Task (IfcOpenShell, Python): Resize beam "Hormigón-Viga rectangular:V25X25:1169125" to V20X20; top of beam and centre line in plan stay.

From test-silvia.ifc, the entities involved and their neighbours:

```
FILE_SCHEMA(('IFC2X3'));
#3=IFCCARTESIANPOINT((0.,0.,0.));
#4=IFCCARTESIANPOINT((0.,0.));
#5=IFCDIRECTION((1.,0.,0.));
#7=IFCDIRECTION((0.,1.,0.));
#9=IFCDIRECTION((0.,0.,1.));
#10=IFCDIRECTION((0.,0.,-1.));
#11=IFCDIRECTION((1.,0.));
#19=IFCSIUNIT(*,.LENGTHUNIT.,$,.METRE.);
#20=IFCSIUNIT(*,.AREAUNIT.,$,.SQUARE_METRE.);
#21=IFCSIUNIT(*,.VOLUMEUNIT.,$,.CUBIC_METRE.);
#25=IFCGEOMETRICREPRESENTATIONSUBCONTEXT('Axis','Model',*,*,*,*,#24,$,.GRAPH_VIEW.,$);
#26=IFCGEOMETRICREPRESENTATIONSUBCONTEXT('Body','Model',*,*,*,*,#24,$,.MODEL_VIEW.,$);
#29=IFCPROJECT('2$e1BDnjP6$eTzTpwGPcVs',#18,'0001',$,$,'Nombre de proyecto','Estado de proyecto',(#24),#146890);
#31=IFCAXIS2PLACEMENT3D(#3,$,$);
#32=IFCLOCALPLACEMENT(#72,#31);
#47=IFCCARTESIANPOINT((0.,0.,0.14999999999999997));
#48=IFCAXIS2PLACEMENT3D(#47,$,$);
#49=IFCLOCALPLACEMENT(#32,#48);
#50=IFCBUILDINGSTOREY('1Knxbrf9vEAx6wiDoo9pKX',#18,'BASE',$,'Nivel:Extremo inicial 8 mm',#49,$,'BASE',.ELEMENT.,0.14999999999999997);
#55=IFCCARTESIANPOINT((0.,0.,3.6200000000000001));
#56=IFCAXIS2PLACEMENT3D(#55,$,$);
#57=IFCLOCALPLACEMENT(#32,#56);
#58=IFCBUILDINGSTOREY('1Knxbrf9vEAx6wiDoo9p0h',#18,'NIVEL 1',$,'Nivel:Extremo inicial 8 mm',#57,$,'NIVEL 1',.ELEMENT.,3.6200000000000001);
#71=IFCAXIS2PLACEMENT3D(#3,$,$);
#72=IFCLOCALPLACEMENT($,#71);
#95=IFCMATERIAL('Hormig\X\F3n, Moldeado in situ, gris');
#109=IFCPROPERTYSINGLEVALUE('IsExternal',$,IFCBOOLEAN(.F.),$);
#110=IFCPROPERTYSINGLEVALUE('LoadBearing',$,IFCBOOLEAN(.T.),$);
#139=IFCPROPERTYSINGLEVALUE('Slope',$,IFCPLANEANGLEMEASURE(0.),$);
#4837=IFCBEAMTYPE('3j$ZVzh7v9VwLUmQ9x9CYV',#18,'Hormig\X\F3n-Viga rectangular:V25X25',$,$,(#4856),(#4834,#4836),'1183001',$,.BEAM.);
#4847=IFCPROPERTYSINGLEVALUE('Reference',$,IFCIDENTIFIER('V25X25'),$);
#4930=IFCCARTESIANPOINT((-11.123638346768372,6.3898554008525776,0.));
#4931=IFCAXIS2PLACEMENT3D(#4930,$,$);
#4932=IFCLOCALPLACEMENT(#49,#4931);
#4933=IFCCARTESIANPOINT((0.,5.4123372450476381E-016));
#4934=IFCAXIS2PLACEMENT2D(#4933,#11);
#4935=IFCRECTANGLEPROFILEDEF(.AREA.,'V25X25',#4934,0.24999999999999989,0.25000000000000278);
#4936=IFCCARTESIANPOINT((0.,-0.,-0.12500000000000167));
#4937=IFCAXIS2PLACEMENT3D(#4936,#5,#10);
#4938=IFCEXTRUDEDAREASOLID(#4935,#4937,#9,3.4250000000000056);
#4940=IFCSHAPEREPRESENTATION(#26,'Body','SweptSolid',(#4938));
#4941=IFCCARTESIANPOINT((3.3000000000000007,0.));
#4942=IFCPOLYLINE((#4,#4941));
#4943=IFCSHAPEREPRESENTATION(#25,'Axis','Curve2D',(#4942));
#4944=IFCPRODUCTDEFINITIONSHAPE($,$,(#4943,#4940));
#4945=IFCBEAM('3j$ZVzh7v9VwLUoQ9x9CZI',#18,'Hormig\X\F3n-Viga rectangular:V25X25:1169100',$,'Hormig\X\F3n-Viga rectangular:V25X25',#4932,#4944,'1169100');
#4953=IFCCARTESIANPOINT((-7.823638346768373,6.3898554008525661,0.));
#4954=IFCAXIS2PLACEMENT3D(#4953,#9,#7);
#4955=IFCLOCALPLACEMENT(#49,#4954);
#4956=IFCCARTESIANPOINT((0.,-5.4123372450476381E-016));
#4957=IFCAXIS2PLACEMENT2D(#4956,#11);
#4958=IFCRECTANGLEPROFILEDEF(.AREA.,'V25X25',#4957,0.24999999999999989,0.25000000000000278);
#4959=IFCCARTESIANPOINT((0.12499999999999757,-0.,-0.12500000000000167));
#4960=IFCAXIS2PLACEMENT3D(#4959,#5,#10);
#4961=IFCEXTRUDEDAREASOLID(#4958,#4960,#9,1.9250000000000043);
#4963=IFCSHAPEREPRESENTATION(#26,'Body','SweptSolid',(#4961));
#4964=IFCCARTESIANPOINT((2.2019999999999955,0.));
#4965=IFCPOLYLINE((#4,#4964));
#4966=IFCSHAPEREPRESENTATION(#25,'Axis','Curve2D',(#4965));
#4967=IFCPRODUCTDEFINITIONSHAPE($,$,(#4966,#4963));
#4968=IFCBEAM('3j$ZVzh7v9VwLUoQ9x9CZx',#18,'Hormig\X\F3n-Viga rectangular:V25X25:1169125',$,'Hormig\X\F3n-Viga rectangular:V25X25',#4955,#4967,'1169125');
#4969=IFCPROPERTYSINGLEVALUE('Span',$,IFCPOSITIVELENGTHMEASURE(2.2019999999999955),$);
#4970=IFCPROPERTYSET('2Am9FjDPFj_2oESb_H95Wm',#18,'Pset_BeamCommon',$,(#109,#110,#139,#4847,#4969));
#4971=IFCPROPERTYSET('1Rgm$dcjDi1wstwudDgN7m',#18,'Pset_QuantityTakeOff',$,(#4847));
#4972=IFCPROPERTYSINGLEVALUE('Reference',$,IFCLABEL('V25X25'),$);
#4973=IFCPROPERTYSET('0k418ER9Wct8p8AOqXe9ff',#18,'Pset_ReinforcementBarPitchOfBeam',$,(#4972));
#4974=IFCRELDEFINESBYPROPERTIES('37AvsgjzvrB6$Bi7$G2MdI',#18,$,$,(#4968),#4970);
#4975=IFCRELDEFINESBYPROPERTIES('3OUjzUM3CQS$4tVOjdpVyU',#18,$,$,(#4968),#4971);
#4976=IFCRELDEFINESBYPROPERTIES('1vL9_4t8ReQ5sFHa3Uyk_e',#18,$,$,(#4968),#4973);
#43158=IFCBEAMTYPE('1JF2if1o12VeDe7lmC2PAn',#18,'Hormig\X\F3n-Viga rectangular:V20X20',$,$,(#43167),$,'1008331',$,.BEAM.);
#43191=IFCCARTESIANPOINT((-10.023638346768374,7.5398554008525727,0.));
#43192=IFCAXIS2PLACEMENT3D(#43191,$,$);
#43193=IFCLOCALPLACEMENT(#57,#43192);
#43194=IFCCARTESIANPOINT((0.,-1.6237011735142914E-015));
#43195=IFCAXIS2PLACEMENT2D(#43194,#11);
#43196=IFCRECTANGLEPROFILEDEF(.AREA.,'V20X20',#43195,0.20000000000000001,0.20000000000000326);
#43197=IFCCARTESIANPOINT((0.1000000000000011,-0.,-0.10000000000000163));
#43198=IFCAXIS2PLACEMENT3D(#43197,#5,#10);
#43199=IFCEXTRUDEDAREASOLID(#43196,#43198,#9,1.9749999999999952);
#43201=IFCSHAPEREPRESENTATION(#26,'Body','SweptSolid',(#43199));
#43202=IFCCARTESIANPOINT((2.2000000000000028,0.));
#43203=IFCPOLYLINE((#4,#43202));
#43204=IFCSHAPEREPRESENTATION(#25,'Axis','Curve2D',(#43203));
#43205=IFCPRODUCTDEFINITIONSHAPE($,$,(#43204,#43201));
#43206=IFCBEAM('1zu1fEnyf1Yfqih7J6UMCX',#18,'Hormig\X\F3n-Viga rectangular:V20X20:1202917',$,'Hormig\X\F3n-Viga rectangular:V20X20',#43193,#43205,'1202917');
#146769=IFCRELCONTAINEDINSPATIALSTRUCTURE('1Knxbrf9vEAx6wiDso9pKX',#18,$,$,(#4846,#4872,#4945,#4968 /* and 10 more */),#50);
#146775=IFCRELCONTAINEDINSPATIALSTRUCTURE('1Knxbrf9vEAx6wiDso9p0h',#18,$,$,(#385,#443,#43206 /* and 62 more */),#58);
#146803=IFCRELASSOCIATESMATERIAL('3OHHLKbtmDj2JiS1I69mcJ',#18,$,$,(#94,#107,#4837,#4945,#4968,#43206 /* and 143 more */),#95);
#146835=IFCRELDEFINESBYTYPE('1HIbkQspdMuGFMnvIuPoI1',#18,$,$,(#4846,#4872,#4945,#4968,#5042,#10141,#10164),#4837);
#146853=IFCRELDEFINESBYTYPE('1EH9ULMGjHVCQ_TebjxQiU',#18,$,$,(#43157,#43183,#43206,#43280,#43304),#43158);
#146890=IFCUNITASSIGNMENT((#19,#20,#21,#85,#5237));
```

```python
import ifcopenshell
import ifcopenshell.api.pset
import ifcopenshell.api.type
import ifcopenshell.util.element
import ifcopenshell.util.representation

model = ifcopenshell.open("test-silvia.ifc")

member = model.by_id(4968)
source = next(p for p in model.by_type("IfcRectangleProfileDef") if p.ProfileName == "V20X20")

body = ifcopenshell.util.representation.get_representation(member, "Model", "Body")
solid = body.Items[0]
old_profile = solid.SweptArea

# Copy the section's sizes but keep this member's own profile position.
profile = ifcopenshell.util.element.copy(model, source)
# Profiles are centred, so shift by half the change in depth to hold the top.
shift = (old_profile.XDim - profile.XDim) / 2
x, y = old_profile.Position.Location.Coordinates
up = (-1.0, 0.0)  # upwards, in the solid's own plane
location = model.createIfcCartesianPoint((x + up[0] * shift, y + up[1] * shift))
profile.Position = model.createIfcAxis2Placement2D(location, old_profile.Position.RefDirection)
solid.SweptArea = profile
if not model.get_total_inverses(old_profile):
    ifcopenshell.util.element.remove_deep2(model, old_profile)

new_type = model.by_id(43158)
ifcopenshell.api.type.assign_type(
    model, related_objects=[member], relating_type=new_type, should_map_representations=False
)
member.Name = member.Name.replace("V25X25", "V20X20")
member.ObjectType = "Hormigón-Viga rectangular:V20X20"
pset = model.by_id(ifcopenshell.util.element.get_pset(member, "Pset_BeamCommon", should_inherit=False)["id"])
ifcopenshell.api.pset.edit_pset(model, pset=pset, properties={"Reference": "V20X20"})
pset = model.by_id(ifcopenshell.util.element.get_pset(member, "Pset_QuantityTakeOff", should_inherit=False)["id"])
ifcopenshell.api.pset.edit_pset(model, pset=pset, properties={"Reference": "V20X20"})
pset = model.by_id(ifcopenshell.util.element.get_pset(member, "Pset_ReinforcementBarPitchOfBeam", should_inherit=False)["id"])
ifcopenshell.api.pset.edit_pset(model, pset=pset, properties={"Reference": "V20X20"})

print(solid.SweptArea)

model.write("test-silvia_updated.ifc")
```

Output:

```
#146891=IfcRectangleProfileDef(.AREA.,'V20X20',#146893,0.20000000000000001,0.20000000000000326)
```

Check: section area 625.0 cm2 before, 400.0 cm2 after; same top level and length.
